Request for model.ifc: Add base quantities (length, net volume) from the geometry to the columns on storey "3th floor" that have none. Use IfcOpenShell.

First a look at what the model holds.

```python
import ifcopenshell
import ifcopenshell.util.element
import ifcopenshell.util.unit

model = ifcopenshell.open("model.ifc")
print(model.schema)
for unit_type in ("LENGTHUNIT", "AREAUNIT", "VOLUMEUNIT"):
    print(unit_type, ifcopenshell.util.unit.calculate_unit_scale(model, unit_type))
storey = next(s for s in model.by_type("IfcBuildingStorey") if s.Name == "3th floor")
columns = [e for e in ifcopenshell.util.element.get_decomposition(storey) if e.is_a("IfcColumn")]
for e in sorted(columns, key=lambda e: e.id()):
    print(e.id(), e.is_a(), e.Name, list(ifcopenshell.util.element.get_psets(e, qtos_only=True)), sep=" | ")
```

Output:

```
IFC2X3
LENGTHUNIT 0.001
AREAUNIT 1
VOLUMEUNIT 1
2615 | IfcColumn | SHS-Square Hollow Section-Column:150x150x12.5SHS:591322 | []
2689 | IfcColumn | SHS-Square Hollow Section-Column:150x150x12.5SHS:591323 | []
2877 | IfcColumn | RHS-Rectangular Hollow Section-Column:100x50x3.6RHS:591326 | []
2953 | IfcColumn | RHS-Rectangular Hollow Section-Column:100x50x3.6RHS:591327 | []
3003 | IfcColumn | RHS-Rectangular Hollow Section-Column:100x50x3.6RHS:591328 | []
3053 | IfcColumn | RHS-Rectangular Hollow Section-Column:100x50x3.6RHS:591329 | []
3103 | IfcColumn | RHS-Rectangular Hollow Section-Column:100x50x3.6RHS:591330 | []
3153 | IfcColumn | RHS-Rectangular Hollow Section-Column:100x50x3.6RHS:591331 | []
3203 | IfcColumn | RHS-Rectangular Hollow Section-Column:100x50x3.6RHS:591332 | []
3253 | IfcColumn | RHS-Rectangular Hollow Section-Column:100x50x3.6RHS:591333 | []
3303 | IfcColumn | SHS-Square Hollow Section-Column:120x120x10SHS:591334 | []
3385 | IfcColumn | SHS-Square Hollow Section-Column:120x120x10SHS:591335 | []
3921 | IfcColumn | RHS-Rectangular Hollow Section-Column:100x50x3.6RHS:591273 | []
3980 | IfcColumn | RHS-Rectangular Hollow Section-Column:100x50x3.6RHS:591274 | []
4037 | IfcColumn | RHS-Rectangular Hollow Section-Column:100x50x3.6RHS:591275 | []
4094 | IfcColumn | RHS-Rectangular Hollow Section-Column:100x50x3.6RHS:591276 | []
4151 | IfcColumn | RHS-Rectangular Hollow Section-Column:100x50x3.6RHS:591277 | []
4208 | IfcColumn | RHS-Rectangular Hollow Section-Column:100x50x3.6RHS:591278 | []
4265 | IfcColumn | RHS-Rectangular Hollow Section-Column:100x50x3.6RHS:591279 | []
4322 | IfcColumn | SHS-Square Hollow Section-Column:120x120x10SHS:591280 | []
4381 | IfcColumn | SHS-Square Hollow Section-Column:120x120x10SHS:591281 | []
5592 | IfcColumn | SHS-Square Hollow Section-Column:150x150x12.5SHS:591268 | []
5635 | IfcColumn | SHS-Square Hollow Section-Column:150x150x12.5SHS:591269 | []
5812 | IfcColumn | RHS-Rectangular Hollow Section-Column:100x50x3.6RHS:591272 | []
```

```python
import ifcopenshell
import ifcopenshell.api.pset
import ifcopenshell.geom
import ifcopenshell.util.element
import ifcopenshell.util.shape
import ifcopenshell.util.unit

model = ifcopenshell.open("model.ifc")
unit_scale = ifcopenshell.util.unit.calculate_unit_scale(model)
volume_scale = ifcopenshell.util.unit.calculate_unit_scale(model, "VOLUMEUNIT")
settings = ifcopenshell.geom.settings()

storey = next(s for s in model.by_type("IfcBuildingStorey") if s.Name == "3th floor")
columns = [e for e in ifcopenshell.util.element.get_decomposition(storey) if e.is_a("IfcColumn")]

for e in sorted(columns, key=lambda e: e.id()):
    if ifcopenshell.util.element.get_psets(e, qtos_only=True, should_inherit=False):
        continue
    # Geometry comes back in metres, in the element's own axes.
    shape = ifcopenshell.geom.create_shape(settings, e)
    values = {
        "Length": ifcopenshell.util.shape.get_z(shape.geometry) / unit_scale,
        "NetVolume": ifcopenshell.util.shape.get_volume(shape.geometry) / volume_scale,
    }
    qto = ifcopenshell.api.pset.add_qto(model, product=e, name="BaseQuantities")
    ifcopenshell.api.pset.edit_qto(model, qto=qto, properties=values)
    print(e.id(), {k: round(v, 3) for k, v in values.items()})

model.write("model_v2.ifc")
```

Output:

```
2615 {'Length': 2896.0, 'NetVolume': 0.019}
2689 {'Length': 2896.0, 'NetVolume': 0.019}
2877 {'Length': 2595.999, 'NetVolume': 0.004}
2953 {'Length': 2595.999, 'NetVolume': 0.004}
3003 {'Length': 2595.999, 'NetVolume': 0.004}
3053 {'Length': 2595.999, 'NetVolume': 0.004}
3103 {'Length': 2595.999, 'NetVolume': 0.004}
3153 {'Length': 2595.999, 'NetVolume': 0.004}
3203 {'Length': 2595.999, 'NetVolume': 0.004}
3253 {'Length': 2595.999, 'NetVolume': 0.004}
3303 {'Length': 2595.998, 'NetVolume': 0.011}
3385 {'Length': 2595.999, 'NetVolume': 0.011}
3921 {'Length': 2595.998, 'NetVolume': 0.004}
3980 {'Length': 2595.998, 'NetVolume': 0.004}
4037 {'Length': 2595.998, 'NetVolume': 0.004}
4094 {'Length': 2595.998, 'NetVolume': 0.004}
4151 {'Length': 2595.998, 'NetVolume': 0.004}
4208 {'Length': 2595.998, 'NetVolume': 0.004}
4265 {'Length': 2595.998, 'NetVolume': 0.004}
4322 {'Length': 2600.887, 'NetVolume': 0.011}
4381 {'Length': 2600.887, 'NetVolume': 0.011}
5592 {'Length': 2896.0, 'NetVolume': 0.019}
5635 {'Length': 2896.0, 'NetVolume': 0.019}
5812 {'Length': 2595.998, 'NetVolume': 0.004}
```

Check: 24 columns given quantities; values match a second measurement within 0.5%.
